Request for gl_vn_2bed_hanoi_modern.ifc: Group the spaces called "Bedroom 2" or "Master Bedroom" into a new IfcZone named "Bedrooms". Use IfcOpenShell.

First a look at what the model holds.

```python
import ifcopenshell

model = ifcopenshell.open("gl_vn_2bed_hanoi_modern.ifc")
print(model.schema)
seen = {}
for space in model.by_type("IfcSpace"):
    seen[space.LongName] = seen.get(space.LongName, 0) + 1
for name, count in sorted(seen.items(), key=str):
    print(count, "x", name)
print("zones:", [z.Name for z in model.by_type("IfcZone")][:20])
```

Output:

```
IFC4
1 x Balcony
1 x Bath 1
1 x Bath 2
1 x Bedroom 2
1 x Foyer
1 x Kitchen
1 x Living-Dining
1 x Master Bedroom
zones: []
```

```python
import ifcopenshell
import ifcopenshell.api.group
import ifcopenshell.api.root

model = ifcopenshell.open("gl_vn_2bed_hanoi_modern.ifc")

names = {"Bedroom 2", "Master Bedroom"}
spaces = [s for s in model.by_type("IfcSpace") if s.LongName in names]

zone = ifcopenshell.api.root.create_entity(model, ifc_class="IfcZone", name="Bedrooms")
ifcopenshell.api.group.assign_group(model, products=spaces, group=zone)
print(len(spaces), "spaces in", zone.Name)

model.write("gl_vn_2bed_hanoi_modern_updated.ifc")
```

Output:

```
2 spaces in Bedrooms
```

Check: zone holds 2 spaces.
